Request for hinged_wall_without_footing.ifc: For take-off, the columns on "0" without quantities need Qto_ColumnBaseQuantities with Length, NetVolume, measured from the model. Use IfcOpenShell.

First a look at what the model holds.

```python
import ifcopenshell
import ifcopenshell.util.element
import ifcopenshell.util.unit

model = ifcopenshell.open("hinged_wall_without_footing.ifc")
print(model.schema)
for unit_type in ("LENGTHUNIT", "AREAUNIT", "VOLUMEUNIT"):
    print(unit_type, ifcopenshell.util.unit.calculate_unit_scale(model, unit_type))
storey = next(s for s in model.by_type("IfcBuildingStorey") if s.Name == "0")
columns = [e for e in ifcopenshell.util.element.get_decomposition(storey) if e.is_a("IfcColumn")]
for e in sorted(columns, key=lambda e: e.id()):
    print(e.id(), e.is_a(), e.Name, list(ifcopenshell.util.element.get_psets(e, qtos_only=True)), sep=" | ")
```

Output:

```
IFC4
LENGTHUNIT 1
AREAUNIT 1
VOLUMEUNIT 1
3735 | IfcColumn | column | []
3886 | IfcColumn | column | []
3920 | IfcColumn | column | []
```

```python
import ifcopenshell
import ifcopenshell.api.pset
import ifcopenshell.geom
import ifcopenshell.util.element
import ifcopenshell.util.shape
import ifcopenshell.util.unit

model = ifcopenshell.open("hinged_wall_without_footing.ifc")
unit_scale = ifcopenshell.util.unit.calculate_unit_scale(model)
volume_scale = ifcopenshell.util.unit.calculate_unit_scale(model, "VOLUMEUNIT")
settings = ifcopenshell.geom.settings()

storey = next(s for s in model.by_type("IfcBuildingStorey") if s.Name == "0")
columns = [e for e in ifcopenshell.util.element.get_decomposition(storey) if e.is_a("IfcColumn")]

for e in sorted(columns, key=lambda e: e.id()):
    if ifcopenshell.util.element.get_psets(e, qtos_only=True, should_inherit=False):
        continue
    # Geometry comes back in metres, in the element's own axes.
    shape = ifcopenshell.geom.create_shape(settings, e)
    values = {
        "Length": ifcopenshell.util.shape.get_z(shape.geometry) / unit_scale,
        "NetVolume": ifcopenshell.util.shape.get_volume(shape.geometry) / volume_scale,
    }
    qto = ifcopenshell.api.pset.add_qto(model, product=e, name="Qto_ColumnBaseQuantities")
    ifcopenshell.api.pset.edit_qto(model, qto=qto, properties=values)
    print(e.id(), {k: round(v, 3) for k, v in values.items()})

model.write("hinged_wall_without_footing-out.ifc")
```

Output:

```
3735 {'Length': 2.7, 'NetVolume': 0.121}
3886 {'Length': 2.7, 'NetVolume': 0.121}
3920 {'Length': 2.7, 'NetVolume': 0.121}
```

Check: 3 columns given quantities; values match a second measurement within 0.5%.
